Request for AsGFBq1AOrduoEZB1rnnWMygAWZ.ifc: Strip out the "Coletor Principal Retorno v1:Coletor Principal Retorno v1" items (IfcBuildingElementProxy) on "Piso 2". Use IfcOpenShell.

First a look at what the model holds.

```python
import ifcopenshell
import ifcopenshell.util.element

model = ifcopenshell.open("AsGFBq1AOrduoEZB1rnnWMygAWZ.ifc")
print(model.schema)
storey = next(s for s in model.by_type("IfcBuildingStorey") if s.Name == "Piso 2")
proxies = [e for e in ifcopenshell.util.element.get_decomposition(storey) if e.is_a("IfcBuildingElementProxy")]
seen = {}
for e in proxies:
    element_type = ifcopenshell.util.element.get_type(e)
    name = element_type.Name if element_type not in (None, e) else None
    seen[name] = seen.get(name, 0) + 1
for name, count in sorted(seen.items(), key=str):
    print(count, "x", name)
```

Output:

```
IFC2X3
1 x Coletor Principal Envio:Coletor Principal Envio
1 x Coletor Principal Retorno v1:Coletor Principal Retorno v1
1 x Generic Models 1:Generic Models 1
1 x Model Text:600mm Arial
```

```python
import ifcopenshell
import ifcopenshell.api.root
import ifcopenshell.util.element

model = ifcopenshell.open("AsGFBq1AOrduoEZB1rnnWMygAWZ.ifc")

storey = next(s for s in model.by_type("IfcBuildingStorey") if s.Name == "Piso 2")
proxies = [e for e in ifcopenshell.util.element.get_decomposition(storey) if e.is_a("IfcBuildingElementProxy")]
targets = [e for e in proxies if (t := ifcopenshell.util.element.get_type(e)) not in (None, e) and t.Name == "Coletor Principal Retorno v1:Coletor Principal Retorno v1"]

for e in targets:
    ifcopenshell.api.root.remove_product(model, product=e)
print(len(targets), "removed")

model.write("AsGFBq1AOrduoEZB1rnnWMygAWZ_rev.ifc")
```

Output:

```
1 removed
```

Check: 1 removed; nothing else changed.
